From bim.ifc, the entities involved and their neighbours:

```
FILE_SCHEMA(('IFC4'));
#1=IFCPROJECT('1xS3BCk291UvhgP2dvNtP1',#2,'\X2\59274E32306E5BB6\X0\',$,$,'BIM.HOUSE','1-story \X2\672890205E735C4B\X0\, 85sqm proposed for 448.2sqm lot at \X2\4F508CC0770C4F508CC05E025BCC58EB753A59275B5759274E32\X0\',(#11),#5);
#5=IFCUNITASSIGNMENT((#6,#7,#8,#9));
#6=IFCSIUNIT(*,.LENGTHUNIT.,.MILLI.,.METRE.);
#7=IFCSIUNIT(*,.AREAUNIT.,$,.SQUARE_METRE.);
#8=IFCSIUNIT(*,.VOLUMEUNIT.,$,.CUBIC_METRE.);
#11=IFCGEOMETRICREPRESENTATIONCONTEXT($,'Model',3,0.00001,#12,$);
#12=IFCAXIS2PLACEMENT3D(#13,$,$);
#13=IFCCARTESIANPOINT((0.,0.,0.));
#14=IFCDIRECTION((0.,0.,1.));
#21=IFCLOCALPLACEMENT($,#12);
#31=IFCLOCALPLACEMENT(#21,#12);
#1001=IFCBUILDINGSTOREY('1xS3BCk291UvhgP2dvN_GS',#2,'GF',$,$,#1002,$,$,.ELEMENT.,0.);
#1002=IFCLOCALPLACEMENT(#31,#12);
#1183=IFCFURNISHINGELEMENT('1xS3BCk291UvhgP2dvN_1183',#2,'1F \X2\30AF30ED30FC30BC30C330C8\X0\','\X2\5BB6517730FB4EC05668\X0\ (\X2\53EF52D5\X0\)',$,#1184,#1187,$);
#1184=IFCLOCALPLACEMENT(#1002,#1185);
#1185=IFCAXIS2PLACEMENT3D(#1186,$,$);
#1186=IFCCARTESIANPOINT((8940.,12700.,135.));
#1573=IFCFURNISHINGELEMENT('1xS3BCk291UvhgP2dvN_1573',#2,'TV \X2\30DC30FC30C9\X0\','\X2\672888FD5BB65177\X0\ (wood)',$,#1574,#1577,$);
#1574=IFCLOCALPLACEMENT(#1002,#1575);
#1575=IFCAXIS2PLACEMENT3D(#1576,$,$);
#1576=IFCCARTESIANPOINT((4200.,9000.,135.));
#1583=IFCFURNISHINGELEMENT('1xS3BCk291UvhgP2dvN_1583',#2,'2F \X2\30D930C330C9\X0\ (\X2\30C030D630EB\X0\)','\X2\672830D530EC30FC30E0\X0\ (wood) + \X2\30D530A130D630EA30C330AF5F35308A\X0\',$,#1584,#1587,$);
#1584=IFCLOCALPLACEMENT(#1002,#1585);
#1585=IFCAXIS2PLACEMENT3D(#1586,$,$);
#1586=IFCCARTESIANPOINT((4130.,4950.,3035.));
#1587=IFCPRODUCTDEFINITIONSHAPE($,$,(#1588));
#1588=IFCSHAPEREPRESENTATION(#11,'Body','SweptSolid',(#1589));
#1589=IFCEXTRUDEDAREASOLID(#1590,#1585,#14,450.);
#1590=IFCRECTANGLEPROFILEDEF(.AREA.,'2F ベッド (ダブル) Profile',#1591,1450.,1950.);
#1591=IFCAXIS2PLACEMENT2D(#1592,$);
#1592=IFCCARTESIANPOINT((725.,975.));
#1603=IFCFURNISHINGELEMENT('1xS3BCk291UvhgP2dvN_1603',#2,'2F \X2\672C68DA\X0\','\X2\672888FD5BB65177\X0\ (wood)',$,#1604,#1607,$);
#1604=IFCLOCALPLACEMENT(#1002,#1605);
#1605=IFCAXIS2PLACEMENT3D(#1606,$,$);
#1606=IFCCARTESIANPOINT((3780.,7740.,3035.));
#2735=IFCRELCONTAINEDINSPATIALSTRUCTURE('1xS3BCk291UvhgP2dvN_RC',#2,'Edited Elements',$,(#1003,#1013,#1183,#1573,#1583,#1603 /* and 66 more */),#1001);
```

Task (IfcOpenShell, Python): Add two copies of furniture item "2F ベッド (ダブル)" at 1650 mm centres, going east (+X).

```python
import numpy as np
import ifcopenshell
import ifcopenshell.api.geometry
import ifcopenshell.api.root
import ifcopenshell.util.element
import ifcopenshell.util.placement
import ifcopenshell.util.unit

model = ifcopenshell.open("bim.ifc")
unit_scale = ifcopenshell.util.unit.calculate_unit_scale(model)


def reuse_history(source, copy):
    """copy_class also copies each property set's owner history, people and application; keep the originals."""
    for rel in copy.IsDefinedBy:
        if rel.is_a("IfcRelDefinesByProperties") and (history := rel.RelatingPropertyDefinition.OwnerHistory):
            rel.RelatingPropertyDefinition.OwnerHistory = source.OwnerHistory
            ifcopenshell.util.element.remove_deep2(model, history)


source = model.by_id(1583)
base = ifcopenshell.util.placement.get_local_placement(source.ObjectPlacement)
step = np.array([1.0, 0.0, 0.0]) * 1.65 / unit_scale

for i in range(1, 3):
    copy = ifcopenshell.api.root.copy_class(model, product=source)
    copy.Representation = ifcopenshell.util.element.copy_deep(
        model, source.Representation, exclude=["IfcGeometricRepresentationContext", "IfcRepresentationMap"]
    )
    reuse_history(source, copy)
    matrix = base.copy()
    matrix[:3, 3] += i * step
    print("added at", matrix[:3, 3].round(3) + 0.0)
    ifcopenshell.api.geometry.edit_object_placement(model, product=copy, matrix=matrix, is_si=False)

model.write("bim-out.ifc")
```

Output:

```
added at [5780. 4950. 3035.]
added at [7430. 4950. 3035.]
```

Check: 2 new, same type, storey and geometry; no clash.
